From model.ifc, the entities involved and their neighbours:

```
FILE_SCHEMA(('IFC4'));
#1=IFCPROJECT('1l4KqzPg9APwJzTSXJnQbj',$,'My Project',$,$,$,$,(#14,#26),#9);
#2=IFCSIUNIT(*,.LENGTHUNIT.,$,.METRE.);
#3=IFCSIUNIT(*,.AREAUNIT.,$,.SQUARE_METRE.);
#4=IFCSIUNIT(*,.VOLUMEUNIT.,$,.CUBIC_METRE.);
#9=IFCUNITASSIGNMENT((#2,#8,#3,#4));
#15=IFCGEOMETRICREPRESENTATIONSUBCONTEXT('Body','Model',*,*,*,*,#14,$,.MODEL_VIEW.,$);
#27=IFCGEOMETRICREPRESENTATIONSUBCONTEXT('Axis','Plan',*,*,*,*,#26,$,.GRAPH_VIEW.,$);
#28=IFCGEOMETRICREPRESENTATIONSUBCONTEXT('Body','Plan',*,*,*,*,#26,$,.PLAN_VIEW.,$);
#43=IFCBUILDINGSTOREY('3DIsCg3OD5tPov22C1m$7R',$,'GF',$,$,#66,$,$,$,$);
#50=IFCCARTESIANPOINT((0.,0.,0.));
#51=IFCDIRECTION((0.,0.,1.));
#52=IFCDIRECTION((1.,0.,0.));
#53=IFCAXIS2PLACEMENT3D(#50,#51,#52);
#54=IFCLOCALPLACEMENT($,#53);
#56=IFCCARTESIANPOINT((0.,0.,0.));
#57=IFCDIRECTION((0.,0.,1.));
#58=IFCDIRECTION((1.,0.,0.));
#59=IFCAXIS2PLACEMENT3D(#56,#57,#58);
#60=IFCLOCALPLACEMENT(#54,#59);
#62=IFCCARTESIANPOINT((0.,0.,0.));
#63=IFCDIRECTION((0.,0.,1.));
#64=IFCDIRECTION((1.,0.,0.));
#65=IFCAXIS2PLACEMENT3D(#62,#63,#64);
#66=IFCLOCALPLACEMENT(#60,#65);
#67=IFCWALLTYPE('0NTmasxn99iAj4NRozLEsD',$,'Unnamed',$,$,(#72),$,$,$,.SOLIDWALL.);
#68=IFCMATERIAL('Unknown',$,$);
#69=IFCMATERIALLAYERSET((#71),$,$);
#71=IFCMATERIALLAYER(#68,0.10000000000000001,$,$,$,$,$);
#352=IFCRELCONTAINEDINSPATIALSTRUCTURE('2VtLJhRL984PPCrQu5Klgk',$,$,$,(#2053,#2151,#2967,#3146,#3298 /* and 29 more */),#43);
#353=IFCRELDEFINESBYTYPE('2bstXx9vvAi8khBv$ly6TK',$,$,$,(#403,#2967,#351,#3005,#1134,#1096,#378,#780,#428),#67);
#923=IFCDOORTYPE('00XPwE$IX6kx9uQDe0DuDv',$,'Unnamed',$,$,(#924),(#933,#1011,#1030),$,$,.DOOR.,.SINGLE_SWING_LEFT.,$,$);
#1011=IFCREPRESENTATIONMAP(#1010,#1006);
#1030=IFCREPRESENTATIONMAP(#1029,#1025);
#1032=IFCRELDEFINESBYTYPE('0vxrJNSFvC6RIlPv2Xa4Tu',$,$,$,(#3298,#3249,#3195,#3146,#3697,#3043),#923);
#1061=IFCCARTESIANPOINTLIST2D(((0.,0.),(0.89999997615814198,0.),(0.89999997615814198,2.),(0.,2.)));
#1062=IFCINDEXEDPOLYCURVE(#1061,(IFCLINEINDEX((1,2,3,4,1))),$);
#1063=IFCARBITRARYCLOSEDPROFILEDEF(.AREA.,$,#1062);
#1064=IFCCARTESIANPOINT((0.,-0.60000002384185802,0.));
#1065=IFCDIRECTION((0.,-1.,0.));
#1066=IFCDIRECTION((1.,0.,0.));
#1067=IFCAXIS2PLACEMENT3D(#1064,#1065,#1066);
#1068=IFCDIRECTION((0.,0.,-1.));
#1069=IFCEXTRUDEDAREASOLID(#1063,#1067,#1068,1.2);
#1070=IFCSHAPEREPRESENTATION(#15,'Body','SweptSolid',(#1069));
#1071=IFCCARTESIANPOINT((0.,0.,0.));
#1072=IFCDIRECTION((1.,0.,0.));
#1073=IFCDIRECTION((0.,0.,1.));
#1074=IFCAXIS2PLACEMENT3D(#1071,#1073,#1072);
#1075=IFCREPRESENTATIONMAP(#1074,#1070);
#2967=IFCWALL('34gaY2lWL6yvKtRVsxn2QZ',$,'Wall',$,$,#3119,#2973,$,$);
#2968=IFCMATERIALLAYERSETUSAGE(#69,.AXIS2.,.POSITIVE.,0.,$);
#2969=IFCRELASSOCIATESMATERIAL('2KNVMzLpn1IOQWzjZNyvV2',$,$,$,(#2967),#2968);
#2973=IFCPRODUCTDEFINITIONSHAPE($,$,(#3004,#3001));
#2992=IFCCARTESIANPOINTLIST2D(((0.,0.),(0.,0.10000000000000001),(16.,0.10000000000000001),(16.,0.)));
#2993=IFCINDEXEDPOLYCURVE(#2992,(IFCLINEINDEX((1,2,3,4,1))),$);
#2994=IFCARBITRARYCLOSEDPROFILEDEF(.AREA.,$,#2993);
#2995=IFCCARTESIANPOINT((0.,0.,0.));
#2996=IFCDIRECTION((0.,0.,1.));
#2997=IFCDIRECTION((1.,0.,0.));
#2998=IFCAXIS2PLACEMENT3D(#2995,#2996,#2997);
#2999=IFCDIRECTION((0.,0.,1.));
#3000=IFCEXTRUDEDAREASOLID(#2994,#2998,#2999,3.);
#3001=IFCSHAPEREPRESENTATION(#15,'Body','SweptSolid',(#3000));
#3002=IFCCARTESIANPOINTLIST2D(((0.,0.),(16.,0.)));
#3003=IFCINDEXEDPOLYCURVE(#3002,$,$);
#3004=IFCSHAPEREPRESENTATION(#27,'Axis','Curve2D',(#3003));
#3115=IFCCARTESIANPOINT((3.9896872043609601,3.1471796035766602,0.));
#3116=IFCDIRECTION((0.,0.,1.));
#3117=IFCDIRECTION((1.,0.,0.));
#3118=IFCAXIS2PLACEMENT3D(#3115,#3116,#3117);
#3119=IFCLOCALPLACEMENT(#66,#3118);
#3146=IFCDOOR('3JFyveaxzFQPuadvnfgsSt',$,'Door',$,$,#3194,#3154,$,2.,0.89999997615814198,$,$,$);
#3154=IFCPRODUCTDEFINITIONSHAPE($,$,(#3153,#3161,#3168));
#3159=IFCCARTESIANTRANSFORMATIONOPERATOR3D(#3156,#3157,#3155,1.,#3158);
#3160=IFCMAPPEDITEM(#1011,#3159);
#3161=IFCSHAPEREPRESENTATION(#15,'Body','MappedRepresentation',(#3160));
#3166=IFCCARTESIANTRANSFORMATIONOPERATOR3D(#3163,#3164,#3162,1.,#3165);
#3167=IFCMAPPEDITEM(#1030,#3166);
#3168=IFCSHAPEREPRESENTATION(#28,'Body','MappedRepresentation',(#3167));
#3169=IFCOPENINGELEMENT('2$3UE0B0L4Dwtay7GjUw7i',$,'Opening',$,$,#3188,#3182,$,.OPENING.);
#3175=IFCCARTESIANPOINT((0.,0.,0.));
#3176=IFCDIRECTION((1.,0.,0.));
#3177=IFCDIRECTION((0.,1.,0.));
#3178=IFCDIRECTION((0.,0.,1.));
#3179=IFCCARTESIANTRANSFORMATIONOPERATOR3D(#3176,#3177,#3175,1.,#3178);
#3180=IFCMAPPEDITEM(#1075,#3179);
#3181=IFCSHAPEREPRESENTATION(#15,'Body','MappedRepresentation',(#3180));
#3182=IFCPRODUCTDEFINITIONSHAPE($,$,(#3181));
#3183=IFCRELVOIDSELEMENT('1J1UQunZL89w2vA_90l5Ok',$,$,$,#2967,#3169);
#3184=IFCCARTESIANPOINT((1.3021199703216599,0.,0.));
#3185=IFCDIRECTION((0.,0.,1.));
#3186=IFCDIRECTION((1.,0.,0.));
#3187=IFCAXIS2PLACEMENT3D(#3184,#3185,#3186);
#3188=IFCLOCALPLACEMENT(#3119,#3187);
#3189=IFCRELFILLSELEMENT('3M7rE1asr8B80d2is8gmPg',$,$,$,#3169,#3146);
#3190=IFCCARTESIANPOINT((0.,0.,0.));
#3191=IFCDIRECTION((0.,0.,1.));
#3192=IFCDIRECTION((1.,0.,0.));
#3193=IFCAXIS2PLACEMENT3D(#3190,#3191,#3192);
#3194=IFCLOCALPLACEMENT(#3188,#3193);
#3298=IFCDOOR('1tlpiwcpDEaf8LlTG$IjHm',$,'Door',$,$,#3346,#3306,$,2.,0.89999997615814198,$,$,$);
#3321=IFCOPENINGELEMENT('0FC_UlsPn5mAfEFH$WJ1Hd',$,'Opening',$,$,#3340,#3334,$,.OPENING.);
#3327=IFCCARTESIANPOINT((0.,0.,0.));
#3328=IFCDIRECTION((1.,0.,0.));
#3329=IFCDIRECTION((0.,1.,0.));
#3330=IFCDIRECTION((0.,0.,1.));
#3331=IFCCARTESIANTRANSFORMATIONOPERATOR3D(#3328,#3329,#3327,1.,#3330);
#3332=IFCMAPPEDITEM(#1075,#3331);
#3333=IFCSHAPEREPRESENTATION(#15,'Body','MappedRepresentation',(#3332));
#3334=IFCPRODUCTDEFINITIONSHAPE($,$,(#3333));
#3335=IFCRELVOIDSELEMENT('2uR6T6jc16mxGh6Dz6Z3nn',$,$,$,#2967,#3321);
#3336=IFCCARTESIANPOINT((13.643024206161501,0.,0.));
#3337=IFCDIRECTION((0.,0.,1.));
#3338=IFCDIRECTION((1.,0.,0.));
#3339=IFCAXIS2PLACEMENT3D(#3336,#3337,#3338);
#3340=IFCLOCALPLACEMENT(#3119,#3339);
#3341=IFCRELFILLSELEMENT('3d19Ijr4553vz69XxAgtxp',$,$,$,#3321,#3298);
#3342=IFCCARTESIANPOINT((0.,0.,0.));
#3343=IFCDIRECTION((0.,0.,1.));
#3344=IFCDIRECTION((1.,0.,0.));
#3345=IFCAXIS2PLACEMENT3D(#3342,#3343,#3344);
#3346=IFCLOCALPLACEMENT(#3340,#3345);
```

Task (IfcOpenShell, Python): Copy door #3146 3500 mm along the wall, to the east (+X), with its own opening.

```python
import ifcopenshell
import ifcopenshell.api.feature
import ifcopenshell.api.geometry
import ifcopenshell.api.root
import ifcopenshell.geom
import ifcopenshell.util.element
import ifcopenshell.util.placement
import ifcopenshell.util.shape
import ifcopenshell.util.unit

model = ifcopenshell.open("model.ifc")
unit_scale = ifcopenshell.util.unit.calculate_unit_scale(model)
settings = ifcopenshell.geom.settings()


def volume(element):
    """Net volume in cubic metres, openings subtracted."""
    shape = ifcopenshell.geom.create_shape(settings, element)
    return ifcopenshell.util.shape.get_volume(shape.geometry)


door = model.by_id(3146)
opening = door.FillsVoids[0].RelatingOpeningElement
wall = opening.VoidsElements[0].RelatingBuildingElement
before = volume(wall)
shift = ifcopenshell.util.placement.get_local_placement(wall.ObjectPlacement)[:3, 0] * 3.5 / unit_scale

# copy_class copies the void relationship, type, container and properties, but no geometry.
new_opening = ifcopenshell.api.root.copy_class(model, product=opening)
new_opening.Representation = ifcopenshell.util.element.copy_deep(
    model, opening.Representation, exclude=["IfcGeometricRepresentationContext", "IfcRepresentationMap"]
)
new_door = ifcopenshell.api.root.copy_class(model, product=door)
new_door.Representation = ifcopenshell.util.element.copy_deep(
    model, door.Representation, exclude=["IfcGeometricRepresentationContext", "IfcRepresentationMap"]
)
ifcopenshell.api.feature.add_filling(model, opening=new_opening, element=new_door)

for old, new in ((opening, new_opening), (door, new_door)):
    matrix = ifcopenshell.util.placement.get_local_placement(old.ObjectPlacement)
    matrix[:3, 3] += shift
    ifcopenshell.api.geometry.edit_object_placement(model, product=new, matrix=matrix, is_si=False)

after = volume(wall)

print(f"wall volume {before:.3f} -> {after:.3f} m3")

model.write("model_rev.ifc")
```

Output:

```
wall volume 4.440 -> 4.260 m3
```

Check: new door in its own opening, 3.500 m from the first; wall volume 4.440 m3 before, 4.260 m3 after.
